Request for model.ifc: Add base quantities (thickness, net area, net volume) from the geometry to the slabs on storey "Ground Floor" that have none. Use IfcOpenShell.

First a look at what the model holds.

```python
import ifcopenshell
import ifcopenshell.util.element
import ifcopenshell.util.unit

model = ifcopenshell.open("model.ifc")
print(model.schema)
for unit_type in ("LENGTHUNIT", "AREAUNIT", "VOLUMEUNIT"):
    print(unit_type, ifcopenshell.util.unit.calculate_unit_scale(model, unit_type))
storey = next(s for s in model.by_type("IfcBuildingStorey") if s.Name == "Ground Floor")
slabs = [e for e in ifcopenshell.util.element.get_decomposition(storey) if e.is_a("IfcSlab")]
for e in sorted(slabs, key=lambda e: e.id()):
    print(e.id(), e.is_a(), e.Name, list(ifcopenshell.util.element.get_psets(e, qtos_only=True)), sep=" | ")
```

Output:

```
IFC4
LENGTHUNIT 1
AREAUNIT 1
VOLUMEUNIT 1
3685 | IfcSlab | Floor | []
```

```python
import ifcopenshell
import ifcopenshell.api.pset
import ifcopenshell.geom
import ifcopenshell.util.element
import ifcopenshell.util.shape
import ifcopenshell.util.unit

model = ifcopenshell.open("model.ifc")
unit_scale = ifcopenshell.util.unit.calculate_unit_scale(model)
area_scale = ifcopenshell.util.unit.calculate_unit_scale(model, "AREAUNIT")
volume_scale = ifcopenshell.util.unit.calculate_unit_scale(model, "VOLUMEUNIT")
settings = ifcopenshell.geom.settings()

storey = next(s for s in model.by_type("IfcBuildingStorey") if s.Name == "Ground Floor")
slabs = [e for e in ifcopenshell.util.element.get_decomposition(storey) if e.is_a("IfcSlab")]

for e in sorted(slabs, key=lambda e: e.id()):
    if ifcopenshell.util.element.get_psets(e, qtos_only=True, should_inherit=False):
        continue
    # Geometry comes back in metres, in the element's own axes.
    shape = ifcopenshell.geom.create_shape(settings, e)
    values = {
        "Width": ifcopenshell.util.shape.get_z(shape.geometry) / unit_scale,
        "NetArea": ifcopenshell.util.shape.get_footprint_area(shape.geometry) / area_scale,
        "NetVolume": ifcopenshell.util.shape.get_volume(shape.geometry) / volume_scale,
    }
    qto = ifcopenshell.api.pset.add_qto(model, product=e, name="Qto_SlabBaseQuantities")
    ifcopenshell.api.pset.edit_qto(model, qto=qto, properties=values)
    print(e.id(), {k: round(v, 3) for k, v in values.items()})

model.write("model_v2.ifc")
```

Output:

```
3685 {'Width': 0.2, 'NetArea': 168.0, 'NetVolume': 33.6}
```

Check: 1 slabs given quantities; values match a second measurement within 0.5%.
